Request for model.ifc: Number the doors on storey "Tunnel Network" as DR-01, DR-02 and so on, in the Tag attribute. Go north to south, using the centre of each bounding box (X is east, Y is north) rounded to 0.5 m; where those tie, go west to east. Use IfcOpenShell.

First a look at what the model holds.

```python
import ifcopenshell
import ifcopenshell.util.element
import ifcopenshell.util.placement

model = ifcopenshell.open("model.ifc")
print(model.schema)
storey = next(s for s in model.by_type("IfcBuildingStorey") if s.Name == "Tunnel Network")
doors = [e for e in ifcopenshell.util.element.get_decomposition(storey) if e.is_a("IfcDoor")]
for e in sorted(doors, key=lambda e: e.id()):
    origin = ifcopenshell.util.placement.get_local_placement(e.ObjectPlacement)[:3, 3]
    print(e.id(), e.Tag, e.Name, origin.round(2) + 0.0, sep=" | ")
```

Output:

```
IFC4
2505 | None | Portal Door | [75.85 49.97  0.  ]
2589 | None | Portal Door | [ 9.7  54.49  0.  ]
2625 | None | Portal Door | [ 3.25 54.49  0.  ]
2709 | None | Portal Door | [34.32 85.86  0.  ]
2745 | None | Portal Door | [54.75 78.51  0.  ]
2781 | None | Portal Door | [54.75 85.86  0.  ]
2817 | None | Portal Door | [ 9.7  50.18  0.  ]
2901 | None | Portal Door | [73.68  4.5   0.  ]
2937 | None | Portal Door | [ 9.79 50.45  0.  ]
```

```python
import ifcopenshell
import ifcopenshell.geom
import ifcopenshell.util.element
import ifcopenshell.util.shape

model = ifcopenshell.open("model.ifc")
settings = ifcopenshell.geom.settings()
settings.set("use-world-coords", True)


def centre(element):
    shape = ifcopenshell.geom.create_shape(settings, element)
    return ifcopenshell.util.shape.get_bbox_centroid(shape.geometry)


storey = next(s for s in model.by_type("IfcBuildingStorey") if s.Name == "Tunnel Network")
doors = [e for e in ifcopenshell.util.element.get_decomposition(storey) if e.is_a("IfcDoor")]

# Insertion points can sit at a corner or the storey origin, so sort by the geometry (in metres).
centres = {e: centre(e) for e in doors}
doors.sort(key=lambda e: (-round(centres[e][1] / 0.5), centres[e][0]))

for i, e in enumerate(doors, start=1):
    number = f"DR-{i:02d}"
    e.Tag = number
    print(e.id(), number)

model.write("model-out.ifc")
```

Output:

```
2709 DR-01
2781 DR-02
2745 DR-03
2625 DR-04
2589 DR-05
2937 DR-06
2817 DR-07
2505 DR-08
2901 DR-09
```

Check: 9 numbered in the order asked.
